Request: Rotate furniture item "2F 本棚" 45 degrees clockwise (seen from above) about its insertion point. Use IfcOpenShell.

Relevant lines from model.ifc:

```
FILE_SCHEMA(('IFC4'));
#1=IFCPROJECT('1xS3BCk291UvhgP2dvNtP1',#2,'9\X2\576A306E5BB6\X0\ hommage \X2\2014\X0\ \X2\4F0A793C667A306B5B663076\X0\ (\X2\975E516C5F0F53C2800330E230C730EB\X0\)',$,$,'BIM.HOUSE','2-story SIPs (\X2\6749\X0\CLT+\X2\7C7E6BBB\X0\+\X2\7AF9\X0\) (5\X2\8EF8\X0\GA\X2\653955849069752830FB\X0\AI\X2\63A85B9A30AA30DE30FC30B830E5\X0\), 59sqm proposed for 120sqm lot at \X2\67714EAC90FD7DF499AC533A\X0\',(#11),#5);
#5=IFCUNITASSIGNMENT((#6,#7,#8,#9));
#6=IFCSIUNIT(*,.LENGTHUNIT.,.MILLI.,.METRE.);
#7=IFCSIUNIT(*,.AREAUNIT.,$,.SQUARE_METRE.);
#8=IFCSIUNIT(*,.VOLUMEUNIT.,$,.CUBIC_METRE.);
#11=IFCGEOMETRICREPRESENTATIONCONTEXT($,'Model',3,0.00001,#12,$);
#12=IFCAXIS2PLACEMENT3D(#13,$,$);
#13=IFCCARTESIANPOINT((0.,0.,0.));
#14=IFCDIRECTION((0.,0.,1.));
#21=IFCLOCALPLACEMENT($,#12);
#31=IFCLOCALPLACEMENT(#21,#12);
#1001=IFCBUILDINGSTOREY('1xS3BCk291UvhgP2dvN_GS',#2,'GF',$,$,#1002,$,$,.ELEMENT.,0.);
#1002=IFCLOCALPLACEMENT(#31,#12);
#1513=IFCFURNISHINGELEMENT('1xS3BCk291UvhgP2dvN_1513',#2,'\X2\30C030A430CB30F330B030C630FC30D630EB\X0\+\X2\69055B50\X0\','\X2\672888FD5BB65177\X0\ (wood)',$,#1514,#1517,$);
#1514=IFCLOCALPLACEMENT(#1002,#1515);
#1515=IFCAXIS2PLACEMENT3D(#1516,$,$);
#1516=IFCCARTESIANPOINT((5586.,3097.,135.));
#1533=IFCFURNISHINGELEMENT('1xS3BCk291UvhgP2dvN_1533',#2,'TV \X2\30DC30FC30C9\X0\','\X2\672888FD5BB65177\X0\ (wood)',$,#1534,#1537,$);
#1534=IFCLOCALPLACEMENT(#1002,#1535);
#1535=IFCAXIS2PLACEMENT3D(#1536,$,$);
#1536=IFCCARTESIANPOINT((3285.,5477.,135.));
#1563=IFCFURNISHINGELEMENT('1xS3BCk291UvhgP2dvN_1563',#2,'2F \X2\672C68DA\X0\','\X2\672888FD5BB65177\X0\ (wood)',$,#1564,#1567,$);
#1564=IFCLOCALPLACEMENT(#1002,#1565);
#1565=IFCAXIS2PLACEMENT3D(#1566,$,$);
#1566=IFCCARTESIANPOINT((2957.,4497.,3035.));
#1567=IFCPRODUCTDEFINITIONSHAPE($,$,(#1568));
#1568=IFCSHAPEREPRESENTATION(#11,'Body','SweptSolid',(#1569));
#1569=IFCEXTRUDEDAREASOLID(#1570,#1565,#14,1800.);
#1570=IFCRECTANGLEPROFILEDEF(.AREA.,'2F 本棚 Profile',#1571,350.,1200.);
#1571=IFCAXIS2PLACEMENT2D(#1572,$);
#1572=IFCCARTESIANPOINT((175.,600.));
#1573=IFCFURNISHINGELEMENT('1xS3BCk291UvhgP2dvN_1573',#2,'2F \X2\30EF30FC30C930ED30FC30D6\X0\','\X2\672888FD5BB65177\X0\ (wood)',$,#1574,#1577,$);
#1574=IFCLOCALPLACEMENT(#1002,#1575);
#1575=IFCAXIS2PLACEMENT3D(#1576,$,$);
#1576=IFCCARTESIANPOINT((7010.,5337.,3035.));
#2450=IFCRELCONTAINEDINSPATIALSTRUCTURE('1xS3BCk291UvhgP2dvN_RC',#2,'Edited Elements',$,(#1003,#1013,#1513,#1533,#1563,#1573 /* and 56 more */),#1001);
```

```python
import ifcopenshell
import ifcopenshell.api.geometry
import ifcopenshell.util.placement

model = ifcopenshell.open("model.ifc")

item = model.by_guid("1xS3BCk291UvhgP2dvN_1563")
matrix = ifcopenshell.util.placement.get_local_placement(item.ObjectPlacement)
matrix = matrix @ ifcopenshell.util.placement.rotation(-45, "Z")
ifcopenshell.api.geometry.edit_object_placement(model, product=item, matrix=matrix, is_si=False)

print(ifcopenshell.util.placement.get_local_placement(item.ObjectPlacement).round(3) + 0.0)

model.write("model_rev.ifc")
```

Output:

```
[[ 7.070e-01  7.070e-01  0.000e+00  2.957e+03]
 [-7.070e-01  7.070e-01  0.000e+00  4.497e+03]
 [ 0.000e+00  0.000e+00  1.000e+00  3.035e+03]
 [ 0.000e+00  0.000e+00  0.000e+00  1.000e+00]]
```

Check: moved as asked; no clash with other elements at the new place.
